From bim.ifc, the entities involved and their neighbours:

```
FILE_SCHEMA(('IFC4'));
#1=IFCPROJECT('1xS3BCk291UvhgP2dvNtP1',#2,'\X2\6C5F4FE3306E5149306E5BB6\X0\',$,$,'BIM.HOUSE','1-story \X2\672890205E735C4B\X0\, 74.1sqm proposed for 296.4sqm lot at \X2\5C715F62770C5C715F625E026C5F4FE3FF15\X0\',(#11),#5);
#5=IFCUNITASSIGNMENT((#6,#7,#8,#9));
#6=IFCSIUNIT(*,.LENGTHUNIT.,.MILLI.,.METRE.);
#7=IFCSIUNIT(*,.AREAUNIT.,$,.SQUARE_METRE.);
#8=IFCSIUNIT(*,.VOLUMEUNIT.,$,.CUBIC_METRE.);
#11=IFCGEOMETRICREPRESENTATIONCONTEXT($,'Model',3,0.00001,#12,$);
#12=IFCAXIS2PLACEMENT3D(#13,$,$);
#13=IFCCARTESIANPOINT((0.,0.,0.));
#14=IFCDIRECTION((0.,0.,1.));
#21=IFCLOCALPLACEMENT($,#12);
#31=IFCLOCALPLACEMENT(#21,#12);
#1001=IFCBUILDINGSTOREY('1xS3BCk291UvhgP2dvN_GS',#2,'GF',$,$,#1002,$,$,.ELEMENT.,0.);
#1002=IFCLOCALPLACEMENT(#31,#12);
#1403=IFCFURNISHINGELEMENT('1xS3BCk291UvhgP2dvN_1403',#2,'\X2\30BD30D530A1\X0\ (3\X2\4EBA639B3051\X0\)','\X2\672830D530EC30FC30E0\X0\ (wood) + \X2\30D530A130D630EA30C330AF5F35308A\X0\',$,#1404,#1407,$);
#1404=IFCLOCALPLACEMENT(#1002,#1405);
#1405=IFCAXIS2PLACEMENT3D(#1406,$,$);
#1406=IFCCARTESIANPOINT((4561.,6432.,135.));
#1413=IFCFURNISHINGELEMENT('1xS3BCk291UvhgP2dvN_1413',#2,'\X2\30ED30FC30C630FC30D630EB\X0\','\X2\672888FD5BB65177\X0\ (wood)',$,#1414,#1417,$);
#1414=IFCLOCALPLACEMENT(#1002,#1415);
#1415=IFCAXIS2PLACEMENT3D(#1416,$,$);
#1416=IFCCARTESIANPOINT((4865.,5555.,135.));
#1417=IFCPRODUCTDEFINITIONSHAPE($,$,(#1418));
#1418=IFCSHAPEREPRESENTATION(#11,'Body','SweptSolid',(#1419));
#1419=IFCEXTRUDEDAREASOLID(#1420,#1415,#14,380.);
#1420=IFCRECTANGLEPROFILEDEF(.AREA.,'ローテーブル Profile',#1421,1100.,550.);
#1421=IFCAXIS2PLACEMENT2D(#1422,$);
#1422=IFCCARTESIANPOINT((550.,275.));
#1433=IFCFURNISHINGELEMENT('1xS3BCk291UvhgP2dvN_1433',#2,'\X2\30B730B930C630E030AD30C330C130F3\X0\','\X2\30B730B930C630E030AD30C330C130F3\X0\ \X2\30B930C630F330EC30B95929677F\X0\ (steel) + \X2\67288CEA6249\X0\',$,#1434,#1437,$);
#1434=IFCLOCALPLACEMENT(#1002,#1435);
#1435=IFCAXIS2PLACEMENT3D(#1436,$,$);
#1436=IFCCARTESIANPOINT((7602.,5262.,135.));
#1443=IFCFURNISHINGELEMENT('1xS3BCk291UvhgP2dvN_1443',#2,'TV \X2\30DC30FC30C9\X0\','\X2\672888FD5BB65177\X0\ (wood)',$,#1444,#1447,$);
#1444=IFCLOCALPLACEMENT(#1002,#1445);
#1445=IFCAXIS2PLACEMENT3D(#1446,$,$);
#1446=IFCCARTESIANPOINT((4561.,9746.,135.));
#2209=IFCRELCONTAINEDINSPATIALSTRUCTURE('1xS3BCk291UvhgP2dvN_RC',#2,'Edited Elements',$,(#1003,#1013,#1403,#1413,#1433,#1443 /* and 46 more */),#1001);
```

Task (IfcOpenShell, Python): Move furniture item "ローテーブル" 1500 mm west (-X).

```python
import ifcopenshell
import ifcopenshell.api.geometry
import ifcopenshell.util.placement
import ifcopenshell.util.unit

model = ifcopenshell.open("bim.ifc")
unit_scale = ifcopenshell.util.unit.calculate_unit_scale(model)

item = model.by_guid("1xS3BCk291UvhgP2dvN_1413")
matrix = ifcopenshell.util.placement.get_local_placement(item.ObjectPlacement)
matrix[0, 3] -= 1.5 / unit_scale
ifcopenshell.api.geometry.edit_object_placement(model, product=item, matrix=matrix, is_si=False)

print(ifcopenshell.util.placement.get_local_placement(item.ObjectPlacement).round(3) + 0.0)

model.write("bim_updated.ifc")
```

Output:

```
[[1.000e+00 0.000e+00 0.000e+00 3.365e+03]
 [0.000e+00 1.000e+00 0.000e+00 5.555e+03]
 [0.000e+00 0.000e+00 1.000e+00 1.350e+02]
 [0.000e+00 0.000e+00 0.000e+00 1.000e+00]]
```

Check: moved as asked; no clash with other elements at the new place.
